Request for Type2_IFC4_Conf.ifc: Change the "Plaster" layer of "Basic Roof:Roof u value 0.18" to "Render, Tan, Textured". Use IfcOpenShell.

First a look at what the model holds.

```python
import ifcopenshell
import ifcopenshell.util.element

model = ifcopenshell.open("Type2_IFC4_Conf.ifc")
print(model.schema)
for layer_set in model.by_type("IfcMaterialLayerSet"):
    if layer_set.LayerSetName == "Basic Roof:Roof u value 0.18":
        for layer in layer_set.MaterialLayers:
            print(layer.id(), layer.Material and layer.Material.Name, layer.LayerThickness, sep=" | ")
        print(len(ifcopenshell.util.element.get_elements_by_material(model, layer_set)), "elements and types use it")
print(sorted(m.Name for m in model.by_type("IfcMaterial") if m.Name)[:60])
```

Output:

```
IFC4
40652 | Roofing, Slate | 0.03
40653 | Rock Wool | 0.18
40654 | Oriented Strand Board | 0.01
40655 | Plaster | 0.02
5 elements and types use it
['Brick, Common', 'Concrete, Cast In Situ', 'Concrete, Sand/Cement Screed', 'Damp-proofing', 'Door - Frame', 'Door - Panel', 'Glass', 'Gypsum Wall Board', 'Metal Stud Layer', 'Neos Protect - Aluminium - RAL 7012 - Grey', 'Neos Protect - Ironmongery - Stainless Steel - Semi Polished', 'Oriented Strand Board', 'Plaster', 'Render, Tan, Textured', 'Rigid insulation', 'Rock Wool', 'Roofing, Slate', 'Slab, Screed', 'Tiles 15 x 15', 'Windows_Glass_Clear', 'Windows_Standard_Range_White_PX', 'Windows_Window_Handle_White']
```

```python
import ifcopenshell
import ifcopenshell.api.material

model = ifcopenshell.open("Type2_IFC4_Conf.ifc")

layer_set = next(s for s in model.by_type("IfcMaterialLayerSet") if s.LayerSetName == "Basic Roof:Roof u value 0.18")
layer = next(l for l in layer_set.MaterialLayers if l.Material and l.Material.Name == "Plaster")
material = next(m for m in model.by_type("IfcMaterial") if m.Name == "Render, Tan, Textured")

# Point this one layer at the other material; renaming the old one would change it everywhere.
ifcopenshell.api.material.edit_layer(model, layer=layer, attributes={"Name": material.Name}, material=material)

print([l.Material.Name if l.Material else None for l in layer_set.MaterialLayers])

model.write("Type2_IFC4_Conf_edited.ifc")
```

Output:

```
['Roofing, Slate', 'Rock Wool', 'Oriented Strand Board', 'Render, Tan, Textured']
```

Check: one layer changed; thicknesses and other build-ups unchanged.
